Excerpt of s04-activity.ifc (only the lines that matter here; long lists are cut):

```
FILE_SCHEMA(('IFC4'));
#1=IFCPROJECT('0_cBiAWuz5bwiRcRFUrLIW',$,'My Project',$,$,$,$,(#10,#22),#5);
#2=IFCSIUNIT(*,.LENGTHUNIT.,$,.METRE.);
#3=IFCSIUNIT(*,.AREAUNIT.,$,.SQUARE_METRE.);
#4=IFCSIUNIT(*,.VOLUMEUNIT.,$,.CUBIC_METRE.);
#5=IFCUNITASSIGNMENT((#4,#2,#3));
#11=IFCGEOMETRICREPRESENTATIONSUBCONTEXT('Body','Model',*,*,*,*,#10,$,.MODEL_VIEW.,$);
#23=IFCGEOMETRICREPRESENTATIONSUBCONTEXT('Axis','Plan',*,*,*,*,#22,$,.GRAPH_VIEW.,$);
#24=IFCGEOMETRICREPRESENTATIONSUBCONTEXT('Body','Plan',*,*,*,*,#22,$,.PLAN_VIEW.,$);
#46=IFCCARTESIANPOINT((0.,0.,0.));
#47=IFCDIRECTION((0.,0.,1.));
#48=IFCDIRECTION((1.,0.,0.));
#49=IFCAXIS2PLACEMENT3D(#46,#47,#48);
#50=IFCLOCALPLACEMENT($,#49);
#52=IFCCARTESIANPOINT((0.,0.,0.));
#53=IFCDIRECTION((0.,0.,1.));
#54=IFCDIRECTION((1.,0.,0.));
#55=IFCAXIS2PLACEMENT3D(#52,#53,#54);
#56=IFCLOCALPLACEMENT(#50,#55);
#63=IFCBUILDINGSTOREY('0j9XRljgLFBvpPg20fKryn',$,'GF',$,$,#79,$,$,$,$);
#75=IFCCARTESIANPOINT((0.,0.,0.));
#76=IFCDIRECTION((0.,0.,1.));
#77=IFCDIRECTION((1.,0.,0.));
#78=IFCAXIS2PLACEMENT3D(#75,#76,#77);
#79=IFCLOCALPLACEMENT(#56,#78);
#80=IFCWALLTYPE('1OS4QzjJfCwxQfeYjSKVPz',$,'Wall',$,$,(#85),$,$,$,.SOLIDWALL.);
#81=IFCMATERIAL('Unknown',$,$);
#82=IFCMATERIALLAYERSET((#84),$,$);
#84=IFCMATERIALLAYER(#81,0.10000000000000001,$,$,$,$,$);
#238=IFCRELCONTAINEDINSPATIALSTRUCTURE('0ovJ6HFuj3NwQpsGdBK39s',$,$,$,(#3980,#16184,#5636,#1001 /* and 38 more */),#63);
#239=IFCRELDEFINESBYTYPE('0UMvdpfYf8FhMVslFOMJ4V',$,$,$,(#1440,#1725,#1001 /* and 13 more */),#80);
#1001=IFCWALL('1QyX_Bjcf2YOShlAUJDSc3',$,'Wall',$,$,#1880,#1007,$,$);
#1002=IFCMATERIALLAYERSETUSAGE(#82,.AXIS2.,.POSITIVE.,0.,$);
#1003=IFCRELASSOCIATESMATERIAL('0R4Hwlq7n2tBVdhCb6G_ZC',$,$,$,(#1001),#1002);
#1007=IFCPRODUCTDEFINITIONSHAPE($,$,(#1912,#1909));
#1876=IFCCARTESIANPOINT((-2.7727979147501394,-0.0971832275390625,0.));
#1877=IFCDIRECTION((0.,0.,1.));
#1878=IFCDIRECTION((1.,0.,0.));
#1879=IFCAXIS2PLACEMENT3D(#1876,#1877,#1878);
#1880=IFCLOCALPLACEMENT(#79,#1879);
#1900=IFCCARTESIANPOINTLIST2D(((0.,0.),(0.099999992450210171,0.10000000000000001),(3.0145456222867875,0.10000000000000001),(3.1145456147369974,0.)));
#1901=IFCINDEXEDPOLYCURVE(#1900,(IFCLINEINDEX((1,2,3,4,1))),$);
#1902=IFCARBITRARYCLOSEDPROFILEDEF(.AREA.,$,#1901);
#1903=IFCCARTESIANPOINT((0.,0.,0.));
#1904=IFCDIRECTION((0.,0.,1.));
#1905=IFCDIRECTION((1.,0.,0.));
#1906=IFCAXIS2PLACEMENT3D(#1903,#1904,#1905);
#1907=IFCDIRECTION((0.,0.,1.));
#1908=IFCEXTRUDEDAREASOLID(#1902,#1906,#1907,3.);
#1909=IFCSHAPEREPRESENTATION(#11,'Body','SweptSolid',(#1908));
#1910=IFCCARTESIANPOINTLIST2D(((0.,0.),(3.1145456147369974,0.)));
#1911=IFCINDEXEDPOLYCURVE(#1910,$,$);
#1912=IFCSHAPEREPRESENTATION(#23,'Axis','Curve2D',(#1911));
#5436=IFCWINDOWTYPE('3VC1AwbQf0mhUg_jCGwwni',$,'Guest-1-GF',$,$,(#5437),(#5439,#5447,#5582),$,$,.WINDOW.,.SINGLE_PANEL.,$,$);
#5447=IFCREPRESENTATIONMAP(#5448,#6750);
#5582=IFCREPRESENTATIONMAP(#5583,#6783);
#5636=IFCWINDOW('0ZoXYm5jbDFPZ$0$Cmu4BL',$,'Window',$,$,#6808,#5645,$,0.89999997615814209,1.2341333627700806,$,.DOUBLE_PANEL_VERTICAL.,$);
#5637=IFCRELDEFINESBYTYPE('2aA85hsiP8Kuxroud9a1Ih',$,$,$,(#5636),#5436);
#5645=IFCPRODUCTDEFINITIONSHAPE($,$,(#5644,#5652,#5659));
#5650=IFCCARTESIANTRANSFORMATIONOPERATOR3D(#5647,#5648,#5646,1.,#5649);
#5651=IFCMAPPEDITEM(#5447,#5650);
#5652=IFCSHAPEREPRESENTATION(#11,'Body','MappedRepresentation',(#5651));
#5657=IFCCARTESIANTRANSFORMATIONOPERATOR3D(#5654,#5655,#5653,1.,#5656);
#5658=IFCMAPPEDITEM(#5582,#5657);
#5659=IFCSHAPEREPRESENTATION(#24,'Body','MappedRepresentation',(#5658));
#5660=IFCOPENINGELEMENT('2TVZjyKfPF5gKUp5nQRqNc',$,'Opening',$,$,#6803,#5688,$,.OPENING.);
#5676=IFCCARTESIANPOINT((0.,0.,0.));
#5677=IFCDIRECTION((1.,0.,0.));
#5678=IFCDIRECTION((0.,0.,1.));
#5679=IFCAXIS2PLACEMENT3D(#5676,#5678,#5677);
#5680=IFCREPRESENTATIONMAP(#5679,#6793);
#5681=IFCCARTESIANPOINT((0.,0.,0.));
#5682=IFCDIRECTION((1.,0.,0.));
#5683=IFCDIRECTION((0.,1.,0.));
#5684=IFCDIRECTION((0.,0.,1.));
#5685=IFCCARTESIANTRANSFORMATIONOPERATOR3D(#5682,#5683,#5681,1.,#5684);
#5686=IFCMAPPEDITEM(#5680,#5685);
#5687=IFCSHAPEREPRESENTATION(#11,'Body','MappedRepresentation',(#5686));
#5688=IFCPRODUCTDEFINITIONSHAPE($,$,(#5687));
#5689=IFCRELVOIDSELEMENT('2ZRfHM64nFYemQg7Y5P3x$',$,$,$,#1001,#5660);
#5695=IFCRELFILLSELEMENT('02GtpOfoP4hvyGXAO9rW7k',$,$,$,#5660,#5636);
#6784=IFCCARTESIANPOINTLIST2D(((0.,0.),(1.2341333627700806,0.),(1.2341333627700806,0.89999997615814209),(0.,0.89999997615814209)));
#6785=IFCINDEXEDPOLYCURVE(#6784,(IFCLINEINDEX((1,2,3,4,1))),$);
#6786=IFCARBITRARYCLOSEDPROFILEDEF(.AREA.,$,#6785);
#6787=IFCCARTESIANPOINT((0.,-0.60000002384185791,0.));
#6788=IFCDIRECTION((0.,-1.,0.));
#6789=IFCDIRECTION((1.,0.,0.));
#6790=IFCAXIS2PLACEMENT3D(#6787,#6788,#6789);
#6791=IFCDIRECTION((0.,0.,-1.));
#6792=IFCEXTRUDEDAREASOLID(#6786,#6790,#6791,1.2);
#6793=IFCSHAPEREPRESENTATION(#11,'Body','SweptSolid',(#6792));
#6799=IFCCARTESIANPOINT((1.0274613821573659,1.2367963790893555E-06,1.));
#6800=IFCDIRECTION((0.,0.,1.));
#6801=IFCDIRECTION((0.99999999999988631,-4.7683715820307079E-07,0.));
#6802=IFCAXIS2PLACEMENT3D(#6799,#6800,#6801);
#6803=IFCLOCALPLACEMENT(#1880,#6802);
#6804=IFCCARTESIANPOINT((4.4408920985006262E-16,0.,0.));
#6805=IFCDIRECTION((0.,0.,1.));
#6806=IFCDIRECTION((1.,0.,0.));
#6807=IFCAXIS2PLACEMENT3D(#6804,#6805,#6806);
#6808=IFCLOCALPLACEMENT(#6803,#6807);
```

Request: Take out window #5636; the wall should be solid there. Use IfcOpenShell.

```python
import ifcopenshell
import ifcopenshell.api.feature
import ifcopenshell.api.root
import ifcopenshell.geom
import ifcopenshell.util.shape

model = ifcopenshell.open("s04-activity.ifc")
settings = ifcopenshell.geom.settings()


def volume(element):
    """Net volume in cubic metres, openings subtracted."""
    shape = ifcopenshell.geom.create_shape(settings, element)
    return ifcopenshell.util.shape.get_volume(shape.geometry)


window = model.by_guid("0ZoXYm5jbDFPZ$0$Cmu4BL")
opening = window.FillsVoids[0].RelatingOpeningElement
wall = opening.VoidsElements[0].RelatingBuildingElement
before = volume(wall)

ifcopenshell.api.root.remove_product(model, product=window)
ifcopenshell.api.feature.remove_feature(model, feature=opening)

after = volume(wall)

print(f"wall volume {before:.3f} -> {after:.3f} m3")

model.write("s04-activity_edited.ifc")
```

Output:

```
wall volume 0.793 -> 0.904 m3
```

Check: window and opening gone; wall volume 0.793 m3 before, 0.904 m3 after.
